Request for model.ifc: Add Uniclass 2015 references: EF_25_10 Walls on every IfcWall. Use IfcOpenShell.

First a look at what the model holds.

```python
import ifcopenshell

model = ifcopenshell.open("model.ifc")
print(model.schema)
print("classifications:", [c.Name for c in model.by_type("IfcClassification")])
for ifc_class in ("IfcDoor", "IfcRoof", "IfcStair", "IfcWall", "IfcWindow"):
    print(ifc_class, len(model.by_type(ifc_class)))
```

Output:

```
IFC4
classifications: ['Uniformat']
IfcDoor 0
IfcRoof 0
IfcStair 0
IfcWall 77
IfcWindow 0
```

```python
import ifcopenshell
import ifcopenshell.api.classification

model = ifcopenshell.open("model.ifc")

system = ifcopenshell.api.classification.add_classification(model, classification="Uniclass 2015")

codes = {
    "IfcWall": ("EF_25_10", "Walls"),
}
for ifc_class, (code, name) in codes.items():
    products = model.by_type(ifc_class)
    ifcopenshell.api.classification.add_reference(
        model, products=products, classification=system, identification=code, name=name
    )
    print(code, len(products))

model.write("model-out.ifc")
```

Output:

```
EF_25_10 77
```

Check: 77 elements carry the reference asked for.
